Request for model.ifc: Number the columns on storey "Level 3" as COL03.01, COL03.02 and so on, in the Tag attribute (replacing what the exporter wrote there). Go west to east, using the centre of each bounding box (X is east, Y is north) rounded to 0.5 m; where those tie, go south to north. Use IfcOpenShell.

First a look at what the model holds.

```python
import ifcopenshell
import ifcopenshell.util.element
import ifcopenshell.util.placement

model = ifcopenshell.open("model.ifc")
print(model.schema)
storey = next(s for s in model.by_type("IfcBuildingStorey") if s.Name == "Level 3")
columns = [e for e in ifcopenshell.util.element.get_decomposition(storey) if e.is_a("IfcColumn")]
for e in sorted(columns, key=lambda e: e.id()):
    origin = ifcopenshell.util.placement.get_local_placement(e.ObjectPlacement)[:3, 3]
    print(e.id(), e.Tag, e.Name, origin.round(2) + 0.0, sep=" | ")
```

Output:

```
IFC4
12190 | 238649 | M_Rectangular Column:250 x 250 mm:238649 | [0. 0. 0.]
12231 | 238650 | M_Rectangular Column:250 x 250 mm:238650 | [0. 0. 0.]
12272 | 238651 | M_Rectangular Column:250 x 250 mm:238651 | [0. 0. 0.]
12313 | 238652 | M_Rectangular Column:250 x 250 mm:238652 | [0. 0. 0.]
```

```python
import ifcopenshell
import ifcopenshell.geom
import ifcopenshell.util.element
import ifcopenshell.util.shape

model = ifcopenshell.open("model.ifc")
settings = ifcopenshell.geom.settings()
settings.set("use-world-coords", True)


def centre(element):
    shape = ifcopenshell.geom.create_shape(settings, element)
    return ifcopenshell.util.shape.get_bbox_centroid(shape.geometry)


storey = next(s for s in model.by_type("IfcBuildingStorey") if s.Name == "Level 3")
columns = [e for e in ifcopenshell.util.element.get_decomposition(storey) if e.is_a("IfcColumn")]

# Insertion points can sit at a corner or the storey origin, so sort by the geometry (in metres).
centres = {e: centre(e) for e in columns}
columns.sort(key=lambda e: (round(centres[e][0] / 0.5), centres[e][1]))

for i, e in enumerate(columns, start=1):
    number = f"COL03.{i:02d}"
    e.Tag = number
    print(e.id(), number)

model.write("model_updated.ifc")
```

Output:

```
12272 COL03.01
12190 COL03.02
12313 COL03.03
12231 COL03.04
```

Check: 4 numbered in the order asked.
